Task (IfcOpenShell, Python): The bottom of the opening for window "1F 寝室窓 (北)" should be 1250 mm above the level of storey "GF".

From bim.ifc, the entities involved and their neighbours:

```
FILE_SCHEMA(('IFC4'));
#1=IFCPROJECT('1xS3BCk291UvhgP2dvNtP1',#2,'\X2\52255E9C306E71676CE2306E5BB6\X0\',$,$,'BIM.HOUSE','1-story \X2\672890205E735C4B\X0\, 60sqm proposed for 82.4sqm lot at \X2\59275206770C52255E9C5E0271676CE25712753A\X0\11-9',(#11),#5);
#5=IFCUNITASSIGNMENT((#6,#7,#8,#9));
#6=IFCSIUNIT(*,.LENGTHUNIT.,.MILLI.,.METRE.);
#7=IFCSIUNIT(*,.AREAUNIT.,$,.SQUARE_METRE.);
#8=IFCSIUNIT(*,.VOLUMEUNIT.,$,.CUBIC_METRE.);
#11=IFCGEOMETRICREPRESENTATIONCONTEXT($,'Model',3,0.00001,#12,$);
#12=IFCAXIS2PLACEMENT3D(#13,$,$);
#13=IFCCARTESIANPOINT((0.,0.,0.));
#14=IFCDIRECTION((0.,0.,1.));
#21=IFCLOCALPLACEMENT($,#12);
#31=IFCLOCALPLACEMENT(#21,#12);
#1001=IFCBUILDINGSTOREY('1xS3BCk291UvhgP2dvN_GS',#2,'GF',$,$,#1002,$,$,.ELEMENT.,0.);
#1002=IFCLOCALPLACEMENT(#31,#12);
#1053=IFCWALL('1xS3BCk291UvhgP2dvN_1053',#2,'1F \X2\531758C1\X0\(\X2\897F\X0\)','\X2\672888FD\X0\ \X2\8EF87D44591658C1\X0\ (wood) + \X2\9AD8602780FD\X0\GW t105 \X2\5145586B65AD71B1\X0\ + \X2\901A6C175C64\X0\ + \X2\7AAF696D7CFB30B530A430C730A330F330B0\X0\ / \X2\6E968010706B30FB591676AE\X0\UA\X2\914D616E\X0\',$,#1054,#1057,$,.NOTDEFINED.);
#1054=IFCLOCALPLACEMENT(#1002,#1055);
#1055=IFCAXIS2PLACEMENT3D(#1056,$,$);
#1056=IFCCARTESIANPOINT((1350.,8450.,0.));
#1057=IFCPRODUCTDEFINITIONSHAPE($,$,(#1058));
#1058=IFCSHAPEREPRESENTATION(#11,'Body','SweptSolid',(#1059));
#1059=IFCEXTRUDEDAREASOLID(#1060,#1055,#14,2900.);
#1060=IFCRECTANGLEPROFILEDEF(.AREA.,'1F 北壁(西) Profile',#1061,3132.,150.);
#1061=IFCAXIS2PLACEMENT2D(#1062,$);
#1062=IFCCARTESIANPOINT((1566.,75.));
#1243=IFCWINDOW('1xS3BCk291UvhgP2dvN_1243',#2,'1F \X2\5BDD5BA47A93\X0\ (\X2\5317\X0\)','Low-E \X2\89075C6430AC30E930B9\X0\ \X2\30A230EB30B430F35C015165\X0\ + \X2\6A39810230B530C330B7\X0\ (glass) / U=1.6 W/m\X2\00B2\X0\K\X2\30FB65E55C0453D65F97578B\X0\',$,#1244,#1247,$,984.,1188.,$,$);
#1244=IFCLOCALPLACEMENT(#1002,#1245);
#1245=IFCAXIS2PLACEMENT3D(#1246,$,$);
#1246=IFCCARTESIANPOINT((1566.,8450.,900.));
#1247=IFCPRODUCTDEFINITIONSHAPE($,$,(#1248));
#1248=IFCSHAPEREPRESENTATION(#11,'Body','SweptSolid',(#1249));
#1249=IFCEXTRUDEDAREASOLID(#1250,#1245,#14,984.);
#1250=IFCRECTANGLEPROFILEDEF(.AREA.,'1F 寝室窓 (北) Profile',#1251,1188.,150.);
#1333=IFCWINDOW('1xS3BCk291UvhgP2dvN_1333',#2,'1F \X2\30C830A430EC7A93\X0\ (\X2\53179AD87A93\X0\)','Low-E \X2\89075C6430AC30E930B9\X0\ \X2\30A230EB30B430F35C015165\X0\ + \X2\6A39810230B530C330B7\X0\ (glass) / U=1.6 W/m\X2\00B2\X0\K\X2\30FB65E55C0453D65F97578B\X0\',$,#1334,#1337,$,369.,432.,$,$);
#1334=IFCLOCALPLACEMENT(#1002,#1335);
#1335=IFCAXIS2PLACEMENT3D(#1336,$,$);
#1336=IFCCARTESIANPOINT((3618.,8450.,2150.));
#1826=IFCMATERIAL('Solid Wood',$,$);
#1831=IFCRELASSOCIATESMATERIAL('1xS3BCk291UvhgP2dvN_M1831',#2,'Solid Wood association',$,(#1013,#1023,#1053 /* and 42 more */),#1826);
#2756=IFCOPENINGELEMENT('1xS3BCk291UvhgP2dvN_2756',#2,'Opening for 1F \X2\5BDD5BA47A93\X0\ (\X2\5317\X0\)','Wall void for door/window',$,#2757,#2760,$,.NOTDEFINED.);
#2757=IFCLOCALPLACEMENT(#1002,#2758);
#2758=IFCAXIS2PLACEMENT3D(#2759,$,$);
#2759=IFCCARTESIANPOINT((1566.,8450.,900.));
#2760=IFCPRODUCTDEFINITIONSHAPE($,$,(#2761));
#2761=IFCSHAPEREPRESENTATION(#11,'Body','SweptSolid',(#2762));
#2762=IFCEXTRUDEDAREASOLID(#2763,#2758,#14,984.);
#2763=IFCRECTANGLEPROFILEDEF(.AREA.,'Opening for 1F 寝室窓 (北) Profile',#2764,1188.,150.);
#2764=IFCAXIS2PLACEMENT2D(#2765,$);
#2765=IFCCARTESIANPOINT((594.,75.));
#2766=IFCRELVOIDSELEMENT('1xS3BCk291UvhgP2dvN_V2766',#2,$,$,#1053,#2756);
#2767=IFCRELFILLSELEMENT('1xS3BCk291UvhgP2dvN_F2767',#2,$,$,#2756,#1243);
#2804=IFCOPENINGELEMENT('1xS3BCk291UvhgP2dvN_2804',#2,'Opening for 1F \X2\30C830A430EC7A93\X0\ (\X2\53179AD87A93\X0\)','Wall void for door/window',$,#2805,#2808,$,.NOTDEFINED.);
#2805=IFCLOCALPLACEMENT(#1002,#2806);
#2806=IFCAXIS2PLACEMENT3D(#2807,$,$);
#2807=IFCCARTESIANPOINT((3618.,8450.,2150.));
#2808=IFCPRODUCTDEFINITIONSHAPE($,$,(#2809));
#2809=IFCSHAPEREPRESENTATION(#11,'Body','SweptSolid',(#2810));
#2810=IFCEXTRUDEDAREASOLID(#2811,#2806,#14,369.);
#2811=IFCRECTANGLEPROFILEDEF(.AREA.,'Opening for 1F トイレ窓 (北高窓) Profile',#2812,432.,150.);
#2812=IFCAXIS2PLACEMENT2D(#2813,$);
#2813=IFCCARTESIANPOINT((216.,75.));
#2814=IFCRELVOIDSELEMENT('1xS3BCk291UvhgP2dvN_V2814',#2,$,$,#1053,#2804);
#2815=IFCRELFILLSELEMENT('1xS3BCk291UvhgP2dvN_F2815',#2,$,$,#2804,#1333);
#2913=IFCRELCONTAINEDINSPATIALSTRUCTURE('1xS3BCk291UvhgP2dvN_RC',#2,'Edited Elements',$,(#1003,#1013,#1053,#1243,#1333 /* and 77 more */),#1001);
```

```python
import numpy as np
import ifcopenshell
import ifcopenshell.api.geometry
import ifcopenshell.geom
import ifcopenshell.util.element
import ifcopenshell.util.placement
import ifcopenshell.util.shape
import ifcopenshell.util.unit

model = ifcopenshell.open("bim.ifc")
unit_scale = ifcopenshell.util.unit.calculate_unit_scale(model)

window = model.by_guid("1xS3BCk291UvhgP2dvN_1243")
opening = window.FillsVoids[0].RelatingOpeningElement
storey = ifcopenshell.util.element.get_container(window, ifc_class="IfcBuildingStorey")
level = ifcopenshell.util.placement.get_local_placement(storey.ObjectPlacement)[2, 3]

# The opening's origin need not be at the sill, so measure its lowest point.
shape = ifcopenshell.geom.create_shape(ifcopenshell.geom.settings(), opening)
bottom = ifcopenshell.util.shape.get_shape_bottom_elevation(shape, shape.geometry) / unit_scale
dz = level + 1250.0 - bottom

shift = np.array([0.0, 0.0, dz])
# The window is not placed relative to its opening, so move both.
for product in (opening, window):
    matrix = ifcopenshell.util.placement.get_local_placement(product.ObjectPlacement)
    matrix[:3, 3] += shift
    ifcopenshell.api.geometry.edit_object_placement(model, product=product, matrix=matrix, is_si=False)

print(f"moved by {dz * unit_scale:+.3f} m")

model.write("bim-out.ifc")
```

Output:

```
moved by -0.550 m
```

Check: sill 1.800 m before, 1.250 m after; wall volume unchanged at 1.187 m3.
